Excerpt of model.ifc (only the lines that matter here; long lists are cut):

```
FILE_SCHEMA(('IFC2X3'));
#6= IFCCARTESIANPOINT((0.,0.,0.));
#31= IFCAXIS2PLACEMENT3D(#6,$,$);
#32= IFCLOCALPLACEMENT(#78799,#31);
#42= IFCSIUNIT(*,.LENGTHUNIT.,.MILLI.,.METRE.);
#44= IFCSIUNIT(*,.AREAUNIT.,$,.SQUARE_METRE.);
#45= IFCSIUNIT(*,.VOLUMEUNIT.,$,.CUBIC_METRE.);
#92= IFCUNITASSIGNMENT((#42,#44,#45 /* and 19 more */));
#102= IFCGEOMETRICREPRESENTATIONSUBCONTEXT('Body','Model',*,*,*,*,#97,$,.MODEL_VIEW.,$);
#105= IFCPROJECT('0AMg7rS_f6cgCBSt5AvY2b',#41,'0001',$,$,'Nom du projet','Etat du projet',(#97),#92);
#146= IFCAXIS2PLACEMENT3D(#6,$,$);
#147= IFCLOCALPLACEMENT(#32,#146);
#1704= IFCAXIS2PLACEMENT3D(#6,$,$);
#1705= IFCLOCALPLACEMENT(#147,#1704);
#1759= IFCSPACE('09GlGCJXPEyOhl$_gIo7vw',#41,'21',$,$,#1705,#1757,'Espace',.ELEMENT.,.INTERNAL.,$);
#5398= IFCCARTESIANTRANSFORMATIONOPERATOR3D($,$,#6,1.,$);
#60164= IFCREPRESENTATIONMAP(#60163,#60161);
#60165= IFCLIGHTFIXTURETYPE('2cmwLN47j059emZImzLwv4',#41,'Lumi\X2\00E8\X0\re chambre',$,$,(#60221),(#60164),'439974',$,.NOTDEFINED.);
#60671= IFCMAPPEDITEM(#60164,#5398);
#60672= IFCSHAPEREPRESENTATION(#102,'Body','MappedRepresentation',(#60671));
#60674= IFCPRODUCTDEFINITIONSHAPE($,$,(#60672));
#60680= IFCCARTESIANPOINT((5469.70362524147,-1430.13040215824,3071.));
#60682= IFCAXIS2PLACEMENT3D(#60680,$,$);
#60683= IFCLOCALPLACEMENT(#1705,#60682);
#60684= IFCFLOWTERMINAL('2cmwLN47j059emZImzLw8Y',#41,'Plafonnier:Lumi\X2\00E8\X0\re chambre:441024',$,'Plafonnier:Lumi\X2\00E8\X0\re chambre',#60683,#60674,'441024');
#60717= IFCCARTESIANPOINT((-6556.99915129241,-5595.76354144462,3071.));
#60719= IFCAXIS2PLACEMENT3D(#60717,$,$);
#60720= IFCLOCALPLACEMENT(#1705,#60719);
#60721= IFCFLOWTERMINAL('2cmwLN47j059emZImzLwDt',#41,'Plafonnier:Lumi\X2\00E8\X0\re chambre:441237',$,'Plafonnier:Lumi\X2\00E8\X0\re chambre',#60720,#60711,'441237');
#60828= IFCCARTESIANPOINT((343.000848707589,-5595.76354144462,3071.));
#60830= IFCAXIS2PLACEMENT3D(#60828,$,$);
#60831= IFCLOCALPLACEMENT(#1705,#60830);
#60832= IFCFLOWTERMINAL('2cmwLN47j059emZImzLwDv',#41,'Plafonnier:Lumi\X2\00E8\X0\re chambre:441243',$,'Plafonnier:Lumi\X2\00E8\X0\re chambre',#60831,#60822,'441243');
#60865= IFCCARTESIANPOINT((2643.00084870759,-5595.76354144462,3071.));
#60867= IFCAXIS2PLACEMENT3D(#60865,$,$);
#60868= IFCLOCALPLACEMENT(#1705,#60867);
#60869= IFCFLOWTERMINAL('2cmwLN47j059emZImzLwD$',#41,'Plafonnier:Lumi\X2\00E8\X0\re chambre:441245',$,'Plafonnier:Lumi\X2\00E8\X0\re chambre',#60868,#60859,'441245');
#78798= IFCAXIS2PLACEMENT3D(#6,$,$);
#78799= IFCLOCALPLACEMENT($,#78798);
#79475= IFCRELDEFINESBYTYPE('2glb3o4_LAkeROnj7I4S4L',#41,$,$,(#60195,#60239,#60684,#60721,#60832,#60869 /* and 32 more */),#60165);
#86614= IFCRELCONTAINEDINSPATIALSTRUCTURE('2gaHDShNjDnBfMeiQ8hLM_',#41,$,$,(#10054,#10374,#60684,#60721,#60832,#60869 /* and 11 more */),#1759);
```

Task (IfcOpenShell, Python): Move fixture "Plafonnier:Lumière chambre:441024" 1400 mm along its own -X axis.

```python
import ifcopenshell
import ifcopenshell.api.geometry
import ifcopenshell.util.placement
import ifcopenshell.util.unit

model = ifcopenshell.open("model.ifc")
unit_scale = ifcopenshell.util.unit.calculate_unit_scale(model)

item = model.by_guid("2cmwLN47j059emZImzLw8Y")
matrix = ifcopenshell.util.placement.get_local_placement(item.ObjectPlacement)
matrix[:3, 3] -= matrix[:3, 0] * 1.4 / unit_scale
ifcopenshell.api.geometry.edit_object_placement(model, product=item, matrix=matrix, is_si=False)

print(ifcopenshell.util.placement.get_local_placement(item.ObjectPlacement).round(3) + 0.0)

model.write("model-out.ifc")
```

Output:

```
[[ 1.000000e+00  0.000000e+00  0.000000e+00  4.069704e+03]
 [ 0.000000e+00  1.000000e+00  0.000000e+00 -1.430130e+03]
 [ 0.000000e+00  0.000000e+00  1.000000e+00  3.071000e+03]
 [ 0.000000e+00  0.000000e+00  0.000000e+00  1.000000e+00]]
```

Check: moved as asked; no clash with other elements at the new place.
